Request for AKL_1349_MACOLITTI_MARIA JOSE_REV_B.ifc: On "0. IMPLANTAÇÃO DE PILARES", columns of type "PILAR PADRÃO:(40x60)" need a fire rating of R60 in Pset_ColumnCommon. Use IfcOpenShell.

First a look at what the model holds.

```python
import ifcopenshell
import ifcopenshell.util.element

model = ifcopenshell.open("AKL_1349_MACOLITTI_MARIA JOSE_REV_B.ifc")
print(model.schema)
storey = next(s for s in model.by_type("IfcBuildingStorey") if s.Name == "0. IMPLANTAÇÃO DE PILARES")
columns = [e for e in ifcopenshell.util.element.get_decomposition(storey) if e.is_a("IfcColumn")]
seen = {}
for e in columns:
    element_type = ifcopenshell.util.element.get_type(e)
    key = (element_type.Name if element_type != e and element_type else None, ifcopenshell.util.element.get_pset(e, "Pset_ColumnCommon", "FireRating"))
    seen[key] = seen.get(key, 0) + 1
for (name, value), count in sorted(seen.items(), key=str):
    print(count, "x", name, "|", value)
```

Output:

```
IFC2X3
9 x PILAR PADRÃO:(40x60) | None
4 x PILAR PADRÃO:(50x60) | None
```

```python
import ifcopenshell
import ifcopenshell.api.pset
import ifcopenshell.util.element

model = ifcopenshell.open("AKL_1349_MACOLITTI_MARIA JOSE_REV_B.ifc")

storey = next(s for s in model.by_type("IfcBuildingStorey") if s.Name == "0. IMPLANTAÇÃO DE PILARES")
columns = [e for e in ifcopenshell.util.element.get_decomposition(storey) if e.is_a("IfcColumn")]

count = 0
for e in columns:
    element_type = ifcopenshell.util.element.get_type(e)
    if element_type in (None, e) or element_type.Name != "PILAR PADRÃO:(40x60)":
        continue
    # add_pset returns the element's existing set when there is one.
    pset = ifcopenshell.api.pset.add_pset(model, product=e, name="Pset_ColumnCommon")
    ifcopenshell.api.pset.edit_pset(model, pset=pset, properties={"FireRating": "R60"})
    count += 1

print(count, "columns updated")

model.write("AKL_1349_MACOLITTI_MARIA JOSE_REV_B_updated.ifc")
```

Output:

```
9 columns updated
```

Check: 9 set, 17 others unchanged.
